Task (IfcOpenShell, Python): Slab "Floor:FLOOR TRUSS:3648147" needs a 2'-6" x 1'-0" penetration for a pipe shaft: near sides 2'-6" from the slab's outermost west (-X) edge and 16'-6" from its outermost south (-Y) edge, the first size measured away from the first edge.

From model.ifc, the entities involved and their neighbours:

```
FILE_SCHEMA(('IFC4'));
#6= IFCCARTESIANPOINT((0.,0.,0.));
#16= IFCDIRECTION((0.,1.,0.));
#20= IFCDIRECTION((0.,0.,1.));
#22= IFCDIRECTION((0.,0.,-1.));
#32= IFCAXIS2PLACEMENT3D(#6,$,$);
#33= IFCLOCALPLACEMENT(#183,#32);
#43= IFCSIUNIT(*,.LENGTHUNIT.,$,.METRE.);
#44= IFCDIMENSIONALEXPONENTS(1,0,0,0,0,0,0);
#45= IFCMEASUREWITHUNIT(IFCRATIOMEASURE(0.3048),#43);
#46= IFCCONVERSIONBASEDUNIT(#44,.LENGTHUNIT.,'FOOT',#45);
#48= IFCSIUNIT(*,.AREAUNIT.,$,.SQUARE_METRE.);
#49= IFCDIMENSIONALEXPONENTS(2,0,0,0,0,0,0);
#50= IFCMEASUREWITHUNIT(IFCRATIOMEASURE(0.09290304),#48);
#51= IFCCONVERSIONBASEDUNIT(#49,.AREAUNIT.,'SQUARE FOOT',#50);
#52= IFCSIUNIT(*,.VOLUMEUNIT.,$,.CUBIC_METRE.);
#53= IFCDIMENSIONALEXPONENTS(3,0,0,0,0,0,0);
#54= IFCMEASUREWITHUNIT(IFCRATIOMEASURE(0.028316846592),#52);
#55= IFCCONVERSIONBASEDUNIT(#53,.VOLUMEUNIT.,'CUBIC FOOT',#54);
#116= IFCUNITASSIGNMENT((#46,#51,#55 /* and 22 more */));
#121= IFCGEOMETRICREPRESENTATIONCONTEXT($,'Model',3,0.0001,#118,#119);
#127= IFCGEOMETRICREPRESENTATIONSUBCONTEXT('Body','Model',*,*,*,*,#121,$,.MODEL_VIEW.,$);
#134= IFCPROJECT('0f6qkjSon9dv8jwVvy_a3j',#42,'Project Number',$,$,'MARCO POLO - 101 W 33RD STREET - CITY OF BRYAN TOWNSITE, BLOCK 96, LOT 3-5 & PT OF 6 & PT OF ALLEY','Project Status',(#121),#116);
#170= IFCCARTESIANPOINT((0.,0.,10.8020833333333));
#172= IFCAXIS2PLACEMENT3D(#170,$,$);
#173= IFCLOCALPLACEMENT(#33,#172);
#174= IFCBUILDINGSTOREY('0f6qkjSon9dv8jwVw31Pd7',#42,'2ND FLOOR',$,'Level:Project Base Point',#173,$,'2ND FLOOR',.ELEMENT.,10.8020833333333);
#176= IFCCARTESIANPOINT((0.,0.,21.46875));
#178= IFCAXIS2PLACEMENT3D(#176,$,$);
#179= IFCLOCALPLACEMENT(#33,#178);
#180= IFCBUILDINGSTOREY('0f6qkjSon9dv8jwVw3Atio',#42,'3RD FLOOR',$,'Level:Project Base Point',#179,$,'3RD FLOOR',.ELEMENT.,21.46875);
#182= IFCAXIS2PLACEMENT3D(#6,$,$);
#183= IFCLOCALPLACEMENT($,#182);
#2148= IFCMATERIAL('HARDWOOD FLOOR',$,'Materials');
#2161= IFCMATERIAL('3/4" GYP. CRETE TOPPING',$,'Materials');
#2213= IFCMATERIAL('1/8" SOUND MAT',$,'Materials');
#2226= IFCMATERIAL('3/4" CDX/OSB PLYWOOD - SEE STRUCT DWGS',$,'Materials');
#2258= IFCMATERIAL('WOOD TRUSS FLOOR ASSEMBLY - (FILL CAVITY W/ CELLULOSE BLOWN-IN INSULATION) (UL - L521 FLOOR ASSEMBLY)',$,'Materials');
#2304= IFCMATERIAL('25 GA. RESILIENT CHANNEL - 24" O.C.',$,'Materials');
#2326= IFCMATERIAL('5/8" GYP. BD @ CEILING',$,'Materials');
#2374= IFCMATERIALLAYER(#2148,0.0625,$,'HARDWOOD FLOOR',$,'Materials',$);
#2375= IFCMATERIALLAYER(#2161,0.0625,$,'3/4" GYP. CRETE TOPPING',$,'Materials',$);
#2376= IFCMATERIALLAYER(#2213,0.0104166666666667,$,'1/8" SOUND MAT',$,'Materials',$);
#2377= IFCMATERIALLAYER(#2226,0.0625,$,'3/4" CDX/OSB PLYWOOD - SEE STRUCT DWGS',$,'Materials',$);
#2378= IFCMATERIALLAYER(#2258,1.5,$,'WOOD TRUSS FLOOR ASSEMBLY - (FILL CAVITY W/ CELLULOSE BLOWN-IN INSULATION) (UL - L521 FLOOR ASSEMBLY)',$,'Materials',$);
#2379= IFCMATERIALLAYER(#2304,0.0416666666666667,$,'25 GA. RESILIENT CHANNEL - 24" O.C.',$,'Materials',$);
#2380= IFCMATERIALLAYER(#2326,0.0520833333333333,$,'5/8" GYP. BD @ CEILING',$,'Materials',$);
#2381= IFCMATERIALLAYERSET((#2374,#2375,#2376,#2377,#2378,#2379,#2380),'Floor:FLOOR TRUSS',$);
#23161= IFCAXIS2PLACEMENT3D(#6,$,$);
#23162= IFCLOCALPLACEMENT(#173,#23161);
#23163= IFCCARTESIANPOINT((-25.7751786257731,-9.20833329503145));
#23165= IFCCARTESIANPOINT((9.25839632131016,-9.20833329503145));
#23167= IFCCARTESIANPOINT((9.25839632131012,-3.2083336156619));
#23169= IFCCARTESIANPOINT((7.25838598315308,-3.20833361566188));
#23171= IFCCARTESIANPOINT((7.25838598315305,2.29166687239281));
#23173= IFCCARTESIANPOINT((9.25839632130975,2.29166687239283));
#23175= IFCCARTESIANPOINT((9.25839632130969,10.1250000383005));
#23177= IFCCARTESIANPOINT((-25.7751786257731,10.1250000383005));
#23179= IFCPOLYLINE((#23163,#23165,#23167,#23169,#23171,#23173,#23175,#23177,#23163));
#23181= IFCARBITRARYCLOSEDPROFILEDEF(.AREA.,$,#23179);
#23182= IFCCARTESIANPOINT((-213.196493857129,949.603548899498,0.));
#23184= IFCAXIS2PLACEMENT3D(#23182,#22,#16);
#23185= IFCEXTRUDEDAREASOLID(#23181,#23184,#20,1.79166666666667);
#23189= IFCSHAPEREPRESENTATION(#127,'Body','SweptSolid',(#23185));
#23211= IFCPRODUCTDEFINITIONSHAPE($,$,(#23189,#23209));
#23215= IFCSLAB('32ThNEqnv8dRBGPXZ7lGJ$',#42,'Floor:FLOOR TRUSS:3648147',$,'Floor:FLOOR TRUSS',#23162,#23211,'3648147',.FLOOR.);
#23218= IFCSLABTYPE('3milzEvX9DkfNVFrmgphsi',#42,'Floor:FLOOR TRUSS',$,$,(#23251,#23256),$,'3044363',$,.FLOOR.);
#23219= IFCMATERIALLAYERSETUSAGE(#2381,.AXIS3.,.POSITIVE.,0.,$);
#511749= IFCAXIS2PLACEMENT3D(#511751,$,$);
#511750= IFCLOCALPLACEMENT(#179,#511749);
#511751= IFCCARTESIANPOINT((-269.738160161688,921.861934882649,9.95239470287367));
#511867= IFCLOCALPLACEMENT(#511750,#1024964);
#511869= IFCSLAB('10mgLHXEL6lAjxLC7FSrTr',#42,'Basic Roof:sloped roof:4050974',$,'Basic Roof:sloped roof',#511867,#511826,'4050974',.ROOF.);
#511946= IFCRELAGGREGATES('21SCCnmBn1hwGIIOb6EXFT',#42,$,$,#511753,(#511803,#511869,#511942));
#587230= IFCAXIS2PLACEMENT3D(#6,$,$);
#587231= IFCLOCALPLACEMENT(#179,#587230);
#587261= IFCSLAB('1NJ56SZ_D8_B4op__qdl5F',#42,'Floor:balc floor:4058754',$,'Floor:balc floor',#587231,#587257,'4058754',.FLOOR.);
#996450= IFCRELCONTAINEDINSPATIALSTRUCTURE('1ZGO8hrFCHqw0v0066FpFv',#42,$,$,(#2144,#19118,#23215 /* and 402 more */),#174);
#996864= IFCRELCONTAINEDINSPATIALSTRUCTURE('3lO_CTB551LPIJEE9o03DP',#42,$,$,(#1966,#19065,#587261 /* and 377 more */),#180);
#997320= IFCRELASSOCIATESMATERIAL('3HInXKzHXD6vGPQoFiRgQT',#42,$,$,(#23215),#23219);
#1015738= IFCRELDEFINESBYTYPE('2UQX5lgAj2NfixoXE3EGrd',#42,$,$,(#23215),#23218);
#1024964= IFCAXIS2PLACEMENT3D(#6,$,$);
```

```python
import numpy as np
import ifcopenshell
import ifcopenshell.api.feature
import ifcopenshell.api.geometry
import ifcopenshell.api.root
import ifcopenshell.geom
import ifcopenshell.util.placement
import ifcopenshell.util.representation
import ifcopenshell.util.shape
import ifcopenshell.util.unit

model = ifcopenshell.open("model.ifc")
unit_scale = ifcopenshell.util.unit.calculate_unit_scale(model)
settings = ifcopenshell.geom.settings()


def volume(element):
    """Net volume in cubic metres, openings subtracted."""
    shape = ifcopenshell.geom.create_shape(settings, element)
    return ifcopenshell.util.shape.get_volume(shape.geometry)


slab = model.by_guid("32ThNEqnv8dRBGPXZ7lGJ$")
before = volume(slab)

# Extent in the slab's own axes, in metres. The edges named are its -X and -Y sides.
slab_shape = ifcopenshell.geom.create_shape(settings, slab)
vertices = ifcopenshell.util.shape.get_vertices(slab_shape.geometry)
x_min, y_min, bottom = vertices.min(axis=0)
top = vertices[:, 2].max()

opening = ifcopenshell.api.root.create_entity(model, ifc_class="IfcOpeningElement", name="Pipe shaft opening", predefined_type="OPENING")
context = ifcopenshell.util.representation.get_context(model, "Model", "Body", "MODEL_VIEW")
width, depth = 0.762, 0.3048
outline = [(0.0, 0.0), (width, 0.0), (width, depth), (0.0, depth), (0.0, 0.0)]
# Overshoot both faces by 50 mm so the cut is clean.
shape = ifcopenshell.api.geometry.add_slab_representation(
    model, context=context, depth=top - bottom + 0.1, polyline=outline
)
ifcopenshell.api.geometry.assign_representation(model, product=opening, representation=shape)

matrix = ifcopenshell.util.placement.get_local_placement(slab.ObjectPlacement)
matrix[:, 3] = matrix @ np.append(np.array([x_min + 0.762, y_min + 5.0292, bottom - 0.05]) / unit_scale, 1.0)
ifcopenshell.api.geometry.edit_object_placement(model, product=opening, matrix=matrix, is_si=False)
ifcopenshell.api.feature.add_feature(model, feature=opening, element=slab)

after = volume(slab)

print(f"slab volume {before:.3f} -> {after:.3f} m3")

model.write("model-out.ifc")
```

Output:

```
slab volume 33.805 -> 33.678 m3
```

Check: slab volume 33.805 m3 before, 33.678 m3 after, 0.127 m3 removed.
